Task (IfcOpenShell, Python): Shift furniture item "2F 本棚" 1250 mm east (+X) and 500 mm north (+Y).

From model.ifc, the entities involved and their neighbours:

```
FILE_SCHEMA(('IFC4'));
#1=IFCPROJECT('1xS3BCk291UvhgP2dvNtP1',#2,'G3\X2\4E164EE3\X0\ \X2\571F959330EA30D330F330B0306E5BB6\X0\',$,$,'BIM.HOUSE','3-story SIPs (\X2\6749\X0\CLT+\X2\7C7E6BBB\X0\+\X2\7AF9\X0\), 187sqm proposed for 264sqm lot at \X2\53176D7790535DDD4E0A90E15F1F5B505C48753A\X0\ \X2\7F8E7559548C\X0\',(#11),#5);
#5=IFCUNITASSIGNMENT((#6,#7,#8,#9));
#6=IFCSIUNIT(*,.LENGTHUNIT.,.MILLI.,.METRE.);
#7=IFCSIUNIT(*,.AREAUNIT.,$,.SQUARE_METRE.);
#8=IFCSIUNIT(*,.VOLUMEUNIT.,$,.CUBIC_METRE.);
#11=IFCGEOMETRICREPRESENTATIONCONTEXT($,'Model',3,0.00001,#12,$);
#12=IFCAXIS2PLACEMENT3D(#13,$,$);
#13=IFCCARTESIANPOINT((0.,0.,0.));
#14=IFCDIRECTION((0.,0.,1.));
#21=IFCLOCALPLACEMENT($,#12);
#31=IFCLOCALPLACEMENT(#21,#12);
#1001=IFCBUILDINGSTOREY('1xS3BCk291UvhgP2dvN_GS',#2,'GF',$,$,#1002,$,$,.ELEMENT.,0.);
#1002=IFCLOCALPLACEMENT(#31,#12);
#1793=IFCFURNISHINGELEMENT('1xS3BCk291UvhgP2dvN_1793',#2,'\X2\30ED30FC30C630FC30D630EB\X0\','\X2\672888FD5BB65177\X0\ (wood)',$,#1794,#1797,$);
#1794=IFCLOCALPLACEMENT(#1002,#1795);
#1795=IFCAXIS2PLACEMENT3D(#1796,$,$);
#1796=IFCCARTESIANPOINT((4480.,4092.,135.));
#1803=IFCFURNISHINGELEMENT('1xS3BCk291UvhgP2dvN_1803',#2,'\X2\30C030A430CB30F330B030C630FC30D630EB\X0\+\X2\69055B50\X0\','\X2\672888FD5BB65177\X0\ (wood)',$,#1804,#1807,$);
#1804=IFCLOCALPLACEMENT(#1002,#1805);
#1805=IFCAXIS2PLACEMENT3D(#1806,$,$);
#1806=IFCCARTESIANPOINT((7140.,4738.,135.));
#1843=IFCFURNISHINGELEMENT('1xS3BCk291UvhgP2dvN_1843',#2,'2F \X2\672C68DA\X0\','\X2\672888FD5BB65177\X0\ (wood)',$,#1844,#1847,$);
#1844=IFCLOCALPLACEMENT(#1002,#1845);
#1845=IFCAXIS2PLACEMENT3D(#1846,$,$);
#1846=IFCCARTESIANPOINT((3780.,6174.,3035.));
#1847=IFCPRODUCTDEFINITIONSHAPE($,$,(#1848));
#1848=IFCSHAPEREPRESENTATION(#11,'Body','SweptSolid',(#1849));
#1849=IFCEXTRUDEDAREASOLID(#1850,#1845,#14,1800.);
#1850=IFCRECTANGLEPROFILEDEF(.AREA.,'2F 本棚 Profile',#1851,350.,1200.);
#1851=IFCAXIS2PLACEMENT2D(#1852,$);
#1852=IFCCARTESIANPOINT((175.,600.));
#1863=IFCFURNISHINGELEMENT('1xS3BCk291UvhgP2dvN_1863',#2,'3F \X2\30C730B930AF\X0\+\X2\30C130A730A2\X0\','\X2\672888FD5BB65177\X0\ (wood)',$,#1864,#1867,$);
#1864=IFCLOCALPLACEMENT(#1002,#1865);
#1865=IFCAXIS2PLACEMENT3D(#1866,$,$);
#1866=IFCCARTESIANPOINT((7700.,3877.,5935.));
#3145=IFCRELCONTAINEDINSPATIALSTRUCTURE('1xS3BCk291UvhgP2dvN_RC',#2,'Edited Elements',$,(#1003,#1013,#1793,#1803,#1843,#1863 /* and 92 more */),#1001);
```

```python
import ifcopenshell
import ifcopenshell.api.geometry
import ifcopenshell.util.placement
import ifcopenshell.util.unit

model = ifcopenshell.open("model.ifc")
unit_scale = ifcopenshell.util.unit.calculate_unit_scale(model)

item = model.by_guid("1xS3BCk291UvhgP2dvN_1843")
matrix = ifcopenshell.util.placement.get_local_placement(item.ObjectPlacement)
matrix[0, 3] += 1.25 / unit_scale
matrix[1, 3] += 0.5 / unit_scale
ifcopenshell.api.geometry.edit_object_placement(model, product=item, matrix=matrix, is_si=False)

print(ifcopenshell.util.placement.get_local_placement(item.ObjectPlacement).round(3) + 0.0)

model.write("model_edited.ifc")
```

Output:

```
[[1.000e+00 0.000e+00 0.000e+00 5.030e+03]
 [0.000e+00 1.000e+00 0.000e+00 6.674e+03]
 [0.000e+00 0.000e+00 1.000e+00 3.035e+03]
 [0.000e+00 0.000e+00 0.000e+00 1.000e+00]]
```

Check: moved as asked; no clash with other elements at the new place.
